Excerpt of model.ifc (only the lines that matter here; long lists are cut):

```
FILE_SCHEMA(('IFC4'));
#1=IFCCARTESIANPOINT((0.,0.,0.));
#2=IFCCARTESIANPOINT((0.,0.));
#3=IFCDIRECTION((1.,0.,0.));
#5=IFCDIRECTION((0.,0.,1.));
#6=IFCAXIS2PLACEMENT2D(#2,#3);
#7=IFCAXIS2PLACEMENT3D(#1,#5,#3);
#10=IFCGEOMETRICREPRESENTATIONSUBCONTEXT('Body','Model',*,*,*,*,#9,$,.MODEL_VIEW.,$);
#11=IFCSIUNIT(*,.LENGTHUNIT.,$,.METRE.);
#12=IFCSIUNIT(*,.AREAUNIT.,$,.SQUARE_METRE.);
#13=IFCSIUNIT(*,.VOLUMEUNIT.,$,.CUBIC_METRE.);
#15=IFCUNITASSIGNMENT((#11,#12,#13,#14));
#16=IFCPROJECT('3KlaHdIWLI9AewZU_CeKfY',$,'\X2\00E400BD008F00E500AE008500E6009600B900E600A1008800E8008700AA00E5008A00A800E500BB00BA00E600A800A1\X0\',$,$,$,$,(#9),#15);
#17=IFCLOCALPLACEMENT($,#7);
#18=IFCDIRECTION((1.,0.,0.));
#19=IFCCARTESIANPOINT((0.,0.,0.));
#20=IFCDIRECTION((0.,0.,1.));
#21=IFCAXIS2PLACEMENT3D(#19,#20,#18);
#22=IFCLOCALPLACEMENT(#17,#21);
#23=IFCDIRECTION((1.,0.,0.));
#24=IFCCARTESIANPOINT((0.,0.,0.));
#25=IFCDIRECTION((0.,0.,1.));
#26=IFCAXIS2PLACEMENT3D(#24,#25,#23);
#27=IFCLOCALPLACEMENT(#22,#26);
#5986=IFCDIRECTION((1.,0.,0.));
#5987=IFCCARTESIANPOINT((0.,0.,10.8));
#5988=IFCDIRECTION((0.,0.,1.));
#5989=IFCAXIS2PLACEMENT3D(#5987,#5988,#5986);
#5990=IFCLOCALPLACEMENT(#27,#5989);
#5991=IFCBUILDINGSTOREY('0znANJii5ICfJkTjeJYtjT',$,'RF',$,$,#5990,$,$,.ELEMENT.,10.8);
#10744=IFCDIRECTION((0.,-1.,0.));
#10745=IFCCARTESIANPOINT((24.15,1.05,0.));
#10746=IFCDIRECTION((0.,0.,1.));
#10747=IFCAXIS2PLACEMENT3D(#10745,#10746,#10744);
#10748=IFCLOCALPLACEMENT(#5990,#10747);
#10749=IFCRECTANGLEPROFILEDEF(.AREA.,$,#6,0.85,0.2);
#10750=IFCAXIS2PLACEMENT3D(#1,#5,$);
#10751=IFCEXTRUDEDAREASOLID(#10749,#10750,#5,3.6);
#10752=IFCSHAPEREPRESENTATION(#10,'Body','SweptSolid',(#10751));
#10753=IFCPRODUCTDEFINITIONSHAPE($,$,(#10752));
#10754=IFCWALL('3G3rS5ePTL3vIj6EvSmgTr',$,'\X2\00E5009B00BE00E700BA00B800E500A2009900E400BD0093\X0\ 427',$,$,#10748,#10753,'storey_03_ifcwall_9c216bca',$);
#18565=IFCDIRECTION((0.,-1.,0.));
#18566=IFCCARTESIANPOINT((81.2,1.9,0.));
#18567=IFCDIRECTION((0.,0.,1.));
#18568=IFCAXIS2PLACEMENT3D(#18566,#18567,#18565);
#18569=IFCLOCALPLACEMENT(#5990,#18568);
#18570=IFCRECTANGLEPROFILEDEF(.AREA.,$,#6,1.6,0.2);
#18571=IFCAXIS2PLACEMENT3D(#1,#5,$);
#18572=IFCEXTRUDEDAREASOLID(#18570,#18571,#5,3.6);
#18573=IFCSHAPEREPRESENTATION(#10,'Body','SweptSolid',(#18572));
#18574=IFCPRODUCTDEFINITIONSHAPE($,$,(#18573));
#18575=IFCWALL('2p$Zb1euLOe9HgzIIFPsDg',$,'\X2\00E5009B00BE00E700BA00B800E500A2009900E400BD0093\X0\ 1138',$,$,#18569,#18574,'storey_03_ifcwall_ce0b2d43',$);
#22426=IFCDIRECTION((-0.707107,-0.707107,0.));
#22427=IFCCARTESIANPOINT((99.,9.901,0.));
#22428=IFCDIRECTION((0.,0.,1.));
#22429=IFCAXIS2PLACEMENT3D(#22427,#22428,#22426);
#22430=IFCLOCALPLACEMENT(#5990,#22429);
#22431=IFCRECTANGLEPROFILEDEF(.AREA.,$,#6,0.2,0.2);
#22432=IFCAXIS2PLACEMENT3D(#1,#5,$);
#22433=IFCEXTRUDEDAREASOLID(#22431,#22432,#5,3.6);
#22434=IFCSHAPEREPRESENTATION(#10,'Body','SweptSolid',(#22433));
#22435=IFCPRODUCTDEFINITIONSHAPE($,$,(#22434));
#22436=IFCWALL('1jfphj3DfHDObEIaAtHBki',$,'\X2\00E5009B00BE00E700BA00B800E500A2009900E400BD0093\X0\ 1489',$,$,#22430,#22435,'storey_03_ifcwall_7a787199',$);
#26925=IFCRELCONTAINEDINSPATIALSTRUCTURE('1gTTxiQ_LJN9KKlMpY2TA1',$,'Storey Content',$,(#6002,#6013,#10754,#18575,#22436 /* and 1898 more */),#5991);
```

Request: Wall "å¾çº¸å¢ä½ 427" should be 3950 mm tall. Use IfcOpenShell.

```python
import ifcopenshell
import ifcopenshell.geom
import ifcopenshell.util.representation
import ifcopenshell.util.shape
import ifcopenshell.util.unit

model = ifcopenshell.open("model.ifc")
unit_scale = ifcopenshell.util.unit.calculate_unit_scale(model)
settings = ifcopenshell.geom.settings()


def volume(element):
    """Net volume in cubic metres, openings subtracted."""
    shape = ifcopenshell.geom.create_shape(settings, element)
    return ifcopenshell.util.shape.get_volume(shape.geometry)


wall = model.by_guid("3G3rS5ePTL3vIj6EvSmgTr")
before = volume(wall)

body = ifcopenshell.util.representation.get_representation(wall, "Model", "Body")
solid = body.Items[0]
old_height = solid.Depth
solid.Depth = 3.95 / unit_scale
after = volume(wall)

print(f"height {old_height:g} -> {solid.Depth:g}, volume {before:.3f} -> {after:.3f} m3")

model.write("model-out.ifc")
```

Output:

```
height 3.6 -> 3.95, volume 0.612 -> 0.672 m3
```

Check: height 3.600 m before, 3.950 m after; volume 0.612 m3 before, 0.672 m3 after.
